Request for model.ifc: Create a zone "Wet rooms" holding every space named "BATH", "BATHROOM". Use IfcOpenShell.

First a look at what the model holds.

```python
import ifcopenshell

model = ifcopenshell.open("model.ifc")
print(model.schema)
seen = {}
for space in model.by_type("IfcSpace"):
    seen[space.LongName] = seen.get(space.LongName, 0) + 1
for name, count in sorted(seen.items(), key=str):
    print(count, "x", name)
print("zones:", [z.Name for z in model.by_type("IfcZone")][:20])
```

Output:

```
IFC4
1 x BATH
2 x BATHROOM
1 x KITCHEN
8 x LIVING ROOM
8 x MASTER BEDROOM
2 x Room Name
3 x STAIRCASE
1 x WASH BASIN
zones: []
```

```python
import ifcopenshell
import ifcopenshell.api.group
import ifcopenshell.api.root

model = ifcopenshell.open("model.ifc")

names = {"BATH", "BATHROOM"}
spaces = [s for s in model.by_type("IfcSpace") if s.LongName in names]

zone = ifcopenshell.api.root.create_entity(model, ifc_class="IfcZone", name="Wet rooms")
ifcopenshell.api.group.assign_group(model, products=spaces, group=zone)
print(len(spaces), "spaces in", zone.Name)

model.write("model_updated.ifc")
```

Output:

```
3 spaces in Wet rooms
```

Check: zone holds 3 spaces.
